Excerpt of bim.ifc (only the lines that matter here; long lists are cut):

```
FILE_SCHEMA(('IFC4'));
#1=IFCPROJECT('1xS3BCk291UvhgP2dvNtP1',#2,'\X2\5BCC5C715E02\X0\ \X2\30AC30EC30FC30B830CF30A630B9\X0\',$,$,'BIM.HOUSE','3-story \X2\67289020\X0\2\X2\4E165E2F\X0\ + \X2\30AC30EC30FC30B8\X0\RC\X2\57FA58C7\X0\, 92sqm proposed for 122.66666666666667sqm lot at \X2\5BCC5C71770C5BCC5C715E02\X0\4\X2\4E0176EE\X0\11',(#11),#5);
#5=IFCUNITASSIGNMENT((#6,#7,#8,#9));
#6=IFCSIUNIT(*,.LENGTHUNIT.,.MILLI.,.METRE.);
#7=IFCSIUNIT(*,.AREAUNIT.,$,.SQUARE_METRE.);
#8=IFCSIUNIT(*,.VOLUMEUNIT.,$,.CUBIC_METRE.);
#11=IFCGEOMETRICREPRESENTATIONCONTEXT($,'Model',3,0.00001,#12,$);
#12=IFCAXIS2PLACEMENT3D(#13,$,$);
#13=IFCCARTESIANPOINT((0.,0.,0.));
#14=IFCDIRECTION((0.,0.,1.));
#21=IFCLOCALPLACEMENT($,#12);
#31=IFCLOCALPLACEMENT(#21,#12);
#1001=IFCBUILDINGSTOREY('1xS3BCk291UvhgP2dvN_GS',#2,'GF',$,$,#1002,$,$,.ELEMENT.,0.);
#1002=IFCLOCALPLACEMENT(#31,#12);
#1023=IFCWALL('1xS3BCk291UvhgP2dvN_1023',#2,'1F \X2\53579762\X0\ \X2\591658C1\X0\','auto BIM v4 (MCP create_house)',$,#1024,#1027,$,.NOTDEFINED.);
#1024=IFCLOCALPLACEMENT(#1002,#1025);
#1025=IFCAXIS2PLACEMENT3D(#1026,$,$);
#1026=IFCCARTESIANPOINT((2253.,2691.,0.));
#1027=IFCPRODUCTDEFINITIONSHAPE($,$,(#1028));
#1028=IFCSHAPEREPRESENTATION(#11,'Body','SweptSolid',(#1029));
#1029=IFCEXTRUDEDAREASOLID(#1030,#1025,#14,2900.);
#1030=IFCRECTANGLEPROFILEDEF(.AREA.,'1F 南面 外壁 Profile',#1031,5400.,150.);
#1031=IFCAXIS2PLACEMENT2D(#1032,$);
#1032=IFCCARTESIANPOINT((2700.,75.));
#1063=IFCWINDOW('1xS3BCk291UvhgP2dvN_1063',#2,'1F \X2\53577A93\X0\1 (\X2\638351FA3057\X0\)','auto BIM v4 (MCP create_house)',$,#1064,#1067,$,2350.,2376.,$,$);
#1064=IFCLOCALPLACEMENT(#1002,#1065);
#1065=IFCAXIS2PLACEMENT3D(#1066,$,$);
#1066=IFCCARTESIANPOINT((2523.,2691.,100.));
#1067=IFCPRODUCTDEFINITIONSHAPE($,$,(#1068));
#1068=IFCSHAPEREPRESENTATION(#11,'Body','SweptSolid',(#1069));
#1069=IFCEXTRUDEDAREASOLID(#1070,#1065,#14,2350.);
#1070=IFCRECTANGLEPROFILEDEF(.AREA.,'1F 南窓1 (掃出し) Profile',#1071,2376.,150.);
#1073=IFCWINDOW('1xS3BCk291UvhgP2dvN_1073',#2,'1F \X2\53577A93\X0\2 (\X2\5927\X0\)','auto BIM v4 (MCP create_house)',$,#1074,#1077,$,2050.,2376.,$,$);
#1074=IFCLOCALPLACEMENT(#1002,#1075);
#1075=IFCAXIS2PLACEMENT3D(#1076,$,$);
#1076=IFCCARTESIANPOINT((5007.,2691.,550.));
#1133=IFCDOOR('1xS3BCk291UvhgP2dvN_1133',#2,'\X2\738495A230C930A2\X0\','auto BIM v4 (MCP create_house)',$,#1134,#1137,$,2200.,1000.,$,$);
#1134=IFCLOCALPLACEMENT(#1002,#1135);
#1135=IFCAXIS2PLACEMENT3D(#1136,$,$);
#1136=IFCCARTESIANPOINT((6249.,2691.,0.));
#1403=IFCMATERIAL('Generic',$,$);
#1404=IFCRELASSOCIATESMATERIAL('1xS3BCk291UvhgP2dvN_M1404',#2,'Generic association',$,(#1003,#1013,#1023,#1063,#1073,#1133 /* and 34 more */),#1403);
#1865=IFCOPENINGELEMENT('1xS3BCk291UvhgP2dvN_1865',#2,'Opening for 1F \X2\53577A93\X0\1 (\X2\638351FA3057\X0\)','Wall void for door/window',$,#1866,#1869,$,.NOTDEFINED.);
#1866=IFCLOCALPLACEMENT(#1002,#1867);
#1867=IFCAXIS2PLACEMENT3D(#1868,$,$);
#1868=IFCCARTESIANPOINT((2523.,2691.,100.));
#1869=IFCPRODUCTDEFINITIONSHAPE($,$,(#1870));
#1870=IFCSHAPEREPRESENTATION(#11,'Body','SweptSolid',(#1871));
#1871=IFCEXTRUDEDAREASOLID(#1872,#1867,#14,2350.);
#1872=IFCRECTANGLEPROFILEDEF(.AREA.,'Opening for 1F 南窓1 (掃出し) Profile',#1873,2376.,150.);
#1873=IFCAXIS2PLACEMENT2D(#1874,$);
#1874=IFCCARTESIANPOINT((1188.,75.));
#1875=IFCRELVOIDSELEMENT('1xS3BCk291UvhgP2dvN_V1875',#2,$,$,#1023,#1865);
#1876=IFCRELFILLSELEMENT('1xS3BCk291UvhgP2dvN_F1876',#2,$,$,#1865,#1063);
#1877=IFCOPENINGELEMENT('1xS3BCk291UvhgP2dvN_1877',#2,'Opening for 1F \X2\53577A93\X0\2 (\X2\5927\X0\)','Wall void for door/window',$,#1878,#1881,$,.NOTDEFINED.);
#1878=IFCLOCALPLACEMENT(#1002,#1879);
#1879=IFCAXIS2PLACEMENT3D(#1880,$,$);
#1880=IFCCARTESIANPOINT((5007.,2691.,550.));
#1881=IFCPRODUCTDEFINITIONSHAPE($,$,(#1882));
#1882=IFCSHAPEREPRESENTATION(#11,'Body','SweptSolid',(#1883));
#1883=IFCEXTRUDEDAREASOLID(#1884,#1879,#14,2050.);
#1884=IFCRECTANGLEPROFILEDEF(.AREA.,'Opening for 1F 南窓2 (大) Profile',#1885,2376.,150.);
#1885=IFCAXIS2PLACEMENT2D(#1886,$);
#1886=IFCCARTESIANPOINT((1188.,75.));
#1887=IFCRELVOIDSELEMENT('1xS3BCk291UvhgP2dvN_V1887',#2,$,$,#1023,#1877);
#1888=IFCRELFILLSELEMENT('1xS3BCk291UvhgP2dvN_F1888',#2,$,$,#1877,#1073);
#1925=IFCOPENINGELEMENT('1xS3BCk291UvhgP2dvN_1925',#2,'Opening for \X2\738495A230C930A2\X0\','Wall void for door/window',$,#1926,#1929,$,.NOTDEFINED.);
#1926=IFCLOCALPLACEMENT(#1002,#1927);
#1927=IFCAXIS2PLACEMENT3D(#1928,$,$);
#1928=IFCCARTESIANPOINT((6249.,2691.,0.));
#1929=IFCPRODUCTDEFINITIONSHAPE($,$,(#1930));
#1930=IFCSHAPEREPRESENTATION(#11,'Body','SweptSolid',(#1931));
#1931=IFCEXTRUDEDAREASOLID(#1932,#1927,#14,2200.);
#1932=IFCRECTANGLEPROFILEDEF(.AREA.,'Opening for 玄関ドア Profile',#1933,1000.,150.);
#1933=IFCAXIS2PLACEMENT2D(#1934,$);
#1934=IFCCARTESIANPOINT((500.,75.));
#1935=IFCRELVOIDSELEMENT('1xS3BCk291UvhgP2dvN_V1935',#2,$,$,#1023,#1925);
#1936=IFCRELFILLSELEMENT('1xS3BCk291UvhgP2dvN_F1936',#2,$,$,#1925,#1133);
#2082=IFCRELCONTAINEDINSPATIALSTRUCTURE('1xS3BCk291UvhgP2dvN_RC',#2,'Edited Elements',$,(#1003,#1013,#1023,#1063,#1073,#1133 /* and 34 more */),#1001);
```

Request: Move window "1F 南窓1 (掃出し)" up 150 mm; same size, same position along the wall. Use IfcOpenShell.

```python
import numpy as np
import ifcopenshell
import ifcopenshell.api.geometry
import ifcopenshell.util.placement
import ifcopenshell.util.unit

model = ifcopenshell.open("bim.ifc")
unit_scale = ifcopenshell.util.unit.calculate_unit_scale(model)

window = model.by_guid("1xS3BCk291UvhgP2dvN_1063")
opening = window.FillsVoids[0].RelatingOpeningElement
dz = 0.15 / unit_scale

shift = np.array([0.0, 0.0, dz])
# The window is not placed relative to its opening, so move both.
for product in (opening, window):
    matrix = ifcopenshell.util.placement.get_local_placement(product.ObjectPlacement)
    matrix[:3, 3] += shift
    ifcopenshell.api.geometry.edit_object_placement(model, product=product, matrix=matrix, is_si=False)

print(f"moved by {dz * unit_scale:+.3f} m")

model.write("bim_edited.ifc")
```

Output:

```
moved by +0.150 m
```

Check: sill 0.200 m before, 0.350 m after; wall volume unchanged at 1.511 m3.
